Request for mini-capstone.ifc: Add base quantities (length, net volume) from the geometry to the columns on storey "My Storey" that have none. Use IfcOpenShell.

First a look at what the model holds.

```python
import ifcopenshell
import ifcopenshell.util.element
import ifcopenshell.util.unit

model = ifcopenshell.open("mini-capstone.ifc")
print(model.schema)
for unit_type in ("LENGTHUNIT", "AREAUNIT", "VOLUMEUNIT"):
    print(unit_type, ifcopenshell.util.unit.calculate_unit_scale(model, unit_type))
storey = next(s for s in model.by_type("IfcBuildingStorey") if s.Name == "My Storey")
columns = [e for e in ifcopenshell.util.element.get_decomposition(storey) if e.is_a("IfcColumn")]
for e in sorted(columns, key=lambda e: e.id()):
    print(e.id(), e.is_a(), e.Name, list(ifcopenshell.util.element.get_psets(e, qtos_only=True)), sep=" | ")
```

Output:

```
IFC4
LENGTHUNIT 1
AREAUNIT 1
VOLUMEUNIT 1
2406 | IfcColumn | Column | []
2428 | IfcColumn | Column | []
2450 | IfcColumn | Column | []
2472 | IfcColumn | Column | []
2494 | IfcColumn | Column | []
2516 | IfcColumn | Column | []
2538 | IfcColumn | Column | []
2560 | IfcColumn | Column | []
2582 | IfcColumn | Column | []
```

```python
import ifcopenshell
import ifcopenshell.api.pset
import ifcopenshell.geom
import ifcopenshell.util.element
import ifcopenshell.util.shape
import ifcopenshell.util.unit

model = ifcopenshell.open("mini-capstone.ifc")
unit_scale = ifcopenshell.util.unit.calculate_unit_scale(model)
volume_scale = ifcopenshell.util.unit.calculate_unit_scale(model, "VOLUMEUNIT")
settings = ifcopenshell.geom.settings()

storey = next(s for s in model.by_type("IfcBuildingStorey") if s.Name == "My Storey")
columns = [e for e in ifcopenshell.util.element.get_decomposition(storey) if e.is_a("IfcColumn")]

for e in sorted(columns, key=lambda e: e.id()):
    if ifcopenshell.util.element.get_psets(e, qtos_only=True, should_inherit=False):
        continue
    # Geometry comes back in metres, in the element's own axes.
    shape = ifcopenshell.geom.create_shape(settings, e)
    values = {
        "Length": ifcopenshell.util.shape.get_z(shape.geometry) / unit_scale,
        "NetVolume": ifcopenshell.util.shape.get_volume(shape.geometry) / volume_scale,
    }
    qto = ifcopenshell.api.pset.add_qto(model, product=e, name="Qto_ColumnBaseQuantities")
    ifcopenshell.api.pset.edit_qto(model, qto=qto, properties=values)
    print(e.id(), {k: round(v, 3) for k, v in values.items()})

model.write("mini-capstone_updated.ifc")
```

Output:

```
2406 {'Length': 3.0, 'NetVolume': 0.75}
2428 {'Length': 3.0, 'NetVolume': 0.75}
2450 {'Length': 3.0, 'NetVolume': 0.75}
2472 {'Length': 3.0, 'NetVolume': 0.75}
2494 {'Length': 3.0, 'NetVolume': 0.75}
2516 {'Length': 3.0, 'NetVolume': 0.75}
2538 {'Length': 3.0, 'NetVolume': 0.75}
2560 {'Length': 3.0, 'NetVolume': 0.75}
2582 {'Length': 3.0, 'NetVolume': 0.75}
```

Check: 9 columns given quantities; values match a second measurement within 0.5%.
